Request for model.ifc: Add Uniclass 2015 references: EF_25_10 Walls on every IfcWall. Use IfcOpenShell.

First a look at what the model holds.

```python
import ifcopenshell

model = ifcopenshell.open("model.ifc")
print(model.schema)
print("classifications:", [c.Name for c in model.by_type("IfcClassification")])
for ifc_class in ("IfcDoor", "IfcRoof", "IfcStair", "IfcWall", "IfcWindow"):
    print(ifc_class, len(model.by_type(ifc_class)))
```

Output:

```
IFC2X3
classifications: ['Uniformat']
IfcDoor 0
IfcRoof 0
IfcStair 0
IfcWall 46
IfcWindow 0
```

```python
import ifcopenshell
import ifcopenshell.api.classification

model = ifcopenshell.open("model.ifc")

# IFC2X3 requires Source and Edition and has no link from the project to the system.
system = model.create_entity("IfcClassification", Source="NBS", Edition="2015", Name="Uniclass 2015")

codes = {
    "IfcWall": ("EF_25_10", "Walls"),
}
for ifc_class, (code, name) in codes.items():
    products = model.by_type(ifc_class)
    ifcopenshell.api.classification.add_reference(
        model, products=products, classification=system, identification=code, name=name
    )
    print(code, len(products))

model.write("model_edited.ifc")
```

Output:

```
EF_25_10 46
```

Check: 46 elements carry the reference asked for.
